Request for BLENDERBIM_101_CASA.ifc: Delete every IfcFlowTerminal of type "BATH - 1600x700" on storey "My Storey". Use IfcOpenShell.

First a look at what the model holds.

```python
import ifcopenshell
import ifcopenshell.util.element

model = ifcopenshell.open("BLENDERBIM_101_CASA.ifc")
print(model.schema)
storey = next(s for s in model.by_type("IfcBuildingStorey") if s.Name == "My Storey")
terminals = [e for e in ifcopenshell.util.element.get_decomposition(storey) if e.is_a("IfcFlowTerminal")]
seen = {}
for e in terminals:
    element_type = ifcopenshell.util.element.get_type(e)
    name = element_type.Name if element_type not in (None, e) else None
    seen[name] = seen.get(name, 0) + 1
for name, count in sorted(seen.items(), key=str):
    print(count, "x", name)
```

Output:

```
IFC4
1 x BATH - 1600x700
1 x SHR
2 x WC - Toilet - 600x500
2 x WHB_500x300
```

```python
import ifcopenshell
import ifcopenshell.api.root
import ifcopenshell.util.element

model = ifcopenshell.open("BLENDERBIM_101_CASA.ifc")

storey = next(s for s in model.by_type("IfcBuildingStorey") if s.Name == "My Storey")
terminals = [e for e in ifcopenshell.util.element.get_decomposition(storey) if e.is_a("IfcFlowTerminal")]
targets = [e for e in terminals if (t := ifcopenshell.util.element.get_type(e)) not in (None, e) and t.Name == "BATH - 1600x700"]

for e in targets:
    ifcopenshell.api.root.remove_product(model, product=e)
print(len(targets), "removed")

model.write("BLENDERBIM_101_CASA-out.ifc")
```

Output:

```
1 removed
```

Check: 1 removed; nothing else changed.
